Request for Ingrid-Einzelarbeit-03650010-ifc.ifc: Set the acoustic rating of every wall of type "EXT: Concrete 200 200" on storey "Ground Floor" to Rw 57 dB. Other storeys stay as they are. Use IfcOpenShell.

First a look at what the model holds.

```python
import ifcopenshell
import ifcopenshell.util.element

model = ifcopenshell.open("Ingrid-Einzelarbeit-03650010-ifc.ifc")
print(model.schema)
storey = next(s for s in model.by_type("IfcBuildingStorey") if s.Name == "Ground Floor")
walls = [e for e in ifcopenshell.util.element.get_decomposition(storey) if e.is_a("IfcWall")]
seen = {}
for e in walls:
    element_type = ifcopenshell.util.element.get_type(e)
    key = (element_type.Name if element_type != e and element_type else None, ifcopenshell.util.element.get_pset(e, "Pset_WallCommon", "AcousticRating"))
    seen[key] = seen.get(key, 0) + 1
for (name, value), count in sorted(seen.items(), key=str):
    print(count, "x", name, "|", value)
```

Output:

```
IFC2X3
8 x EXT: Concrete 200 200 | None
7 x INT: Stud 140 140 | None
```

```python
import ifcopenshell
import ifcopenshell.api.pset
import ifcopenshell.util.element

model = ifcopenshell.open("Ingrid-Einzelarbeit-03650010-ifc.ifc")

storey = next(s for s in model.by_type("IfcBuildingStorey") if s.Name == "Ground Floor")
walls = [e for e in ifcopenshell.util.element.get_decomposition(storey) if e.is_a("IfcWall")]

count = 0
for e in walls:
    element_type = ifcopenshell.util.element.get_type(e)
    if element_type in (None, e) or element_type.Name != "EXT: Concrete 200 200":
        continue
    # add_pset returns the element's existing set when there is one.
    pset = ifcopenshell.api.pset.add_pset(model, product=e, name="Pset_WallCommon")
    ifcopenshell.api.pset.edit_pset(model, pset=pset, properties={"AcousticRating": "Rw 57 dB"})
    count += 1

print(count, "walls updated")

model.write("Ingrid-Einzelarbeit-03650010-ifc_v2.ifc")
```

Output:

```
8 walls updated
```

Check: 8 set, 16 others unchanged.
